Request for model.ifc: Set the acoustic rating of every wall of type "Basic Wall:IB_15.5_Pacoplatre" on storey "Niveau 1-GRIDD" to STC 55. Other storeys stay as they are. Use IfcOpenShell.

First a look at what the model holds.

```python
import ifcopenshell
import ifcopenshell.util.element

model = ifcopenshell.open("model.ifc")
print(model.schema)
storey = next(s for s in model.by_type("IfcBuildingStorey") if s.Name == "Niveau 1-GRIDD")
walls = [e for e in ifcopenshell.util.element.get_decomposition(storey) if e.is_a("IfcWall")]
seen = {}
for e in walls:
    element_type = ifcopenshell.util.element.get_type(e)
    key = (element_type.Name if element_type != e and element_type else None, ifcopenshell.util.element.get_pset(e, "Pset_WallCommon", "AcousticRating"))
    seen[key] = seen.get(key, 0) + 1
for (name, value), count in sorted(seen.items(), key=str):
    print(count, "x", name, "|", value)
```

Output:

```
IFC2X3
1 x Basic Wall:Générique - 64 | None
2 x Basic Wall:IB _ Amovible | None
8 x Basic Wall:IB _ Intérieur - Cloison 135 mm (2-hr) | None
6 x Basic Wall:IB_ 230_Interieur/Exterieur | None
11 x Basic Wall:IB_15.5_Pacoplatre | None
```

```python
import ifcopenshell
import ifcopenshell.api.pset
import ifcopenshell.util.element

model = ifcopenshell.open("model.ifc")

storey = next(s for s in model.by_type("IfcBuildingStorey") if s.Name == "Niveau 1-GRIDD")
walls = [e for e in ifcopenshell.util.element.get_decomposition(storey) if e.is_a("IfcWall")]

count = 0
for e in walls:
    element_type = ifcopenshell.util.element.get_type(e)
    if element_type in (None, e) or element_type.Name != "Basic Wall:IB_15.5_Pacoplatre":
        continue
    # add_pset returns the element's existing set when there is one.
    pset = ifcopenshell.api.pset.add_pset(model, product=e, name="Pset_WallCommon")
    ifcopenshell.api.pset.edit_pset(model, pset=pset, properties={"AcousticRating": "STC 55"})
    count += 1

print(count, "walls updated")

model.write("model_updated.ifc")
```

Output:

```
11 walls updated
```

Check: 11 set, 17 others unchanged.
